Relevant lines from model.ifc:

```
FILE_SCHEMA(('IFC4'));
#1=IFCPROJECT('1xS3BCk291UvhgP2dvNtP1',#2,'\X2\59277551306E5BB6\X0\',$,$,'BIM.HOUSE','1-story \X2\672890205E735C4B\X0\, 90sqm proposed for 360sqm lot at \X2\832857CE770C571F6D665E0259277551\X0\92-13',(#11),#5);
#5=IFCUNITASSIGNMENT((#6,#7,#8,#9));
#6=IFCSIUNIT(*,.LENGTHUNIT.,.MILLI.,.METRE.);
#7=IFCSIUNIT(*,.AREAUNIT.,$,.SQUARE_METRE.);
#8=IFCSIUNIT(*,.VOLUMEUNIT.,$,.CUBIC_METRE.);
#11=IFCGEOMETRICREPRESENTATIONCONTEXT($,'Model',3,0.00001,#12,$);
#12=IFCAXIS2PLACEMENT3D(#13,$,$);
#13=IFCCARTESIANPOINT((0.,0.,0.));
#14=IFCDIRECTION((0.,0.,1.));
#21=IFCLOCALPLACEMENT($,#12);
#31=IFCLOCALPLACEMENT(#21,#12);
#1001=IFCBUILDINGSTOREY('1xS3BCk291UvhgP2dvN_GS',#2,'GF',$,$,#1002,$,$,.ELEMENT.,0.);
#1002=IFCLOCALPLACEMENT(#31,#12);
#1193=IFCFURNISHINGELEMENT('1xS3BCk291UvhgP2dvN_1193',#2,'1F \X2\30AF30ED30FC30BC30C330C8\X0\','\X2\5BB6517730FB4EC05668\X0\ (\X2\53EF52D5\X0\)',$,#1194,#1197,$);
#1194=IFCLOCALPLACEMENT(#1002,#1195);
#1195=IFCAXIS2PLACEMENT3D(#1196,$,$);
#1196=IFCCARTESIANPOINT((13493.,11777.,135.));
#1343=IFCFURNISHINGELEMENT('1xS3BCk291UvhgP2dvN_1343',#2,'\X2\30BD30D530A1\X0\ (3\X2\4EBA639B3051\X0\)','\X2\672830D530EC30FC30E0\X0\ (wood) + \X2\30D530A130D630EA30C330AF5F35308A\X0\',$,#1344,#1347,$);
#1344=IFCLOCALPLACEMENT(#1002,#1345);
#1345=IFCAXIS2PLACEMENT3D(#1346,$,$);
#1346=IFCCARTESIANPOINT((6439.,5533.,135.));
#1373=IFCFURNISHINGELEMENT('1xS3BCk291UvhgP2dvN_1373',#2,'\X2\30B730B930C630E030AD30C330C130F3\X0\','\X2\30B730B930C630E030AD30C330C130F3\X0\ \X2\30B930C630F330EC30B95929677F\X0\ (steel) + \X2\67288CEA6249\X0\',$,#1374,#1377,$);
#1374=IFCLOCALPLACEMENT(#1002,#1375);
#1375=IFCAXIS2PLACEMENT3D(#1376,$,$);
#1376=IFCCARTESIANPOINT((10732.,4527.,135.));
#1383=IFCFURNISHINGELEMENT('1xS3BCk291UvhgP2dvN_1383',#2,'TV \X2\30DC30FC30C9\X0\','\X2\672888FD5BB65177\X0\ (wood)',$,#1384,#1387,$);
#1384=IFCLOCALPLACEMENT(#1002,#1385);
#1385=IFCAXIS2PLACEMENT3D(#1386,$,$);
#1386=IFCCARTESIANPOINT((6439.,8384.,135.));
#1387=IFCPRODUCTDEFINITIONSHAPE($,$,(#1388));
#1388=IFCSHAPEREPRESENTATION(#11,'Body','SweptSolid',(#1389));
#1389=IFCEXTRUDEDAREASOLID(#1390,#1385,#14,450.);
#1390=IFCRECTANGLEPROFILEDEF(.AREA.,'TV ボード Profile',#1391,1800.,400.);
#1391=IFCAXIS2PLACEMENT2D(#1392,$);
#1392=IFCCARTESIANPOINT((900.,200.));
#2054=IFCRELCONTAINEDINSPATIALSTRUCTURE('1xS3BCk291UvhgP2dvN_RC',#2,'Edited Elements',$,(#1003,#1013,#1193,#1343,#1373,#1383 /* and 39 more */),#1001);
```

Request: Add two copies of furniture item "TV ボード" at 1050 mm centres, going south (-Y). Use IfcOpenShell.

```python
import numpy as np
import ifcopenshell
import ifcopenshell.api.geometry
import ifcopenshell.api.root
import ifcopenshell.util.element
import ifcopenshell.util.placement
import ifcopenshell.util.unit

model = ifcopenshell.open("model.ifc")
unit_scale = ifcopenshell.util.unit.calculate_unit_scale(model)


def reuse_history(source, copy):
    """copy_class also copies each property set's owner history, people and application; keep the originals."""
    for rel in copy.IsDefinedBy:
        if rel.is_a("IfcRelDefinesByProperties") and (history := rel.RelatingPropertyDefinition.OwnerHistory):
            rel.RelatingPropertyDefinition.OwnerHistory = source.OwnerHistory
            ifcopenshell.util.element.remove_deep2(model, history)


source = model.by_guid("1xS3BCk291UvhgP2dvN_1383")
base = ifcopenshell.util.placement.get_local_placement(source.ObjectPlacement)
step = np.array([0.0, -1.0, 0.0]) * 1.05 / unit_scale

for i in range(1, 3):
    copy = ifcopenshell.api.root.copy_class(model, product=source)
    copy.Representation = ifcopenshell.util.element.copy_deep(
        model, source.Representation, exclude=["IfcGeometricRepresentationContext", "IfcRepresentationMap"]
    )
    reuse_history(source, copy)
    matrix = base.copy()
    matrix[:3, 3] += i * step
    print("added at", matrix[:3, 3].round(3) + 0.0)
    ifcopenshell.api.geometry.edit_object_placement(model, product=copy, matrix=matrix, is_si=False)

model.write("model_rev.ifc")
```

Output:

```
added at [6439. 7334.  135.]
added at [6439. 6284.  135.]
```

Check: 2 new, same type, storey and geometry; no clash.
